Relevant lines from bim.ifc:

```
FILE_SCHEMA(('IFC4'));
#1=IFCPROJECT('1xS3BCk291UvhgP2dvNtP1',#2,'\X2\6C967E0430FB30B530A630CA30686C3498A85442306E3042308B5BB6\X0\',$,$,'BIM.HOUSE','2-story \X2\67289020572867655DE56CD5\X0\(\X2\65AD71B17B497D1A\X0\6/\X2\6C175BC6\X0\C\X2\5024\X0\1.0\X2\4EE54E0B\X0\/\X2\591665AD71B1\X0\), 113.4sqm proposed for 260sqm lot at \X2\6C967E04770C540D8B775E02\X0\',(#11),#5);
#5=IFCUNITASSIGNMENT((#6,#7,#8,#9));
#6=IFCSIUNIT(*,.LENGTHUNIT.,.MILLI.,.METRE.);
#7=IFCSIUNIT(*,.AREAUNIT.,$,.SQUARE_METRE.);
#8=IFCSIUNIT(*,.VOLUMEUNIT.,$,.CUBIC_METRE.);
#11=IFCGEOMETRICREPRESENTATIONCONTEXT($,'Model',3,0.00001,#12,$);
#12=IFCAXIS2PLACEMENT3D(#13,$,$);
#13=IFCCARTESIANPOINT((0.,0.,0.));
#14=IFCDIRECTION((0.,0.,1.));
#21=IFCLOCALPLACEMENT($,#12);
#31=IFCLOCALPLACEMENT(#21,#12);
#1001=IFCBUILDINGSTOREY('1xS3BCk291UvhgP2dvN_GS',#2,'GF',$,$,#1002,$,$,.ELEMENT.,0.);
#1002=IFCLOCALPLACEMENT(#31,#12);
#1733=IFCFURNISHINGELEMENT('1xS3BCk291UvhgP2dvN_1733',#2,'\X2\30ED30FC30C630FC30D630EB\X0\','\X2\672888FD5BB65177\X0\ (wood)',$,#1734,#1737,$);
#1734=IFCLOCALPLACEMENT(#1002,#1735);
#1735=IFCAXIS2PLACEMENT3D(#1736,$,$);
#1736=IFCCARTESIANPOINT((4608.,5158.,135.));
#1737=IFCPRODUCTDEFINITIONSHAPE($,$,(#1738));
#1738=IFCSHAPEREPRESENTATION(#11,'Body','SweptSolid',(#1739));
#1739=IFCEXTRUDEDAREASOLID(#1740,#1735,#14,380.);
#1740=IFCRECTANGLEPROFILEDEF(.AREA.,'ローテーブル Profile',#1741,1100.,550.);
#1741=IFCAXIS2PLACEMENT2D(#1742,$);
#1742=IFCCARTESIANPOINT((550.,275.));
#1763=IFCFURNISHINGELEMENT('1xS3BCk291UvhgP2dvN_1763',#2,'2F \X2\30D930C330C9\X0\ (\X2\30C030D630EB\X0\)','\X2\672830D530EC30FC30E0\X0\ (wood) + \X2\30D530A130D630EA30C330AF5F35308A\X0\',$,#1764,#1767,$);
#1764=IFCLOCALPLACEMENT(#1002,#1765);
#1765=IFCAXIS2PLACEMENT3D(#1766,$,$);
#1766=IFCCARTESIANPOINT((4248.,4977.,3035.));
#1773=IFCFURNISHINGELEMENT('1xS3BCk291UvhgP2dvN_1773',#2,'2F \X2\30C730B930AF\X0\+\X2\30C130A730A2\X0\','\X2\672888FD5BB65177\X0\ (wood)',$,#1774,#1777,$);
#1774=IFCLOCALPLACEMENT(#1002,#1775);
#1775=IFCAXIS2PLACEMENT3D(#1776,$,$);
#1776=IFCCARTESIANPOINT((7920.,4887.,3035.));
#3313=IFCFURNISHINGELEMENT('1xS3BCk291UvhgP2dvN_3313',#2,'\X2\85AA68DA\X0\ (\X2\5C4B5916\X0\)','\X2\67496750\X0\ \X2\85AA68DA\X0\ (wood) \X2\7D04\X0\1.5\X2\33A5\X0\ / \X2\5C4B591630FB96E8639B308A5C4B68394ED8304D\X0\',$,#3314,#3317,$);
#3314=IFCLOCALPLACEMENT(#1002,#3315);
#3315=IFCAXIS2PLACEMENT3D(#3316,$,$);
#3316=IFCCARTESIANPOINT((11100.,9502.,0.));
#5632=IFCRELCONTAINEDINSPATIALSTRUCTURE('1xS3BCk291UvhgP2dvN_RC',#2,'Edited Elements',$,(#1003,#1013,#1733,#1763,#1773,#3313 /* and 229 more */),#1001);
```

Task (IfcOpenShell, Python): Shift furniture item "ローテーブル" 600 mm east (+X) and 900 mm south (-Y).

```python
import ifcopenshell
import ifcopenshell.api.geometry
import ifcopenshell.util.placement
import ifcopenshell.util.unit

model = ifcopenshell.open("bim.ifc")
unit_scale = ifcopenshell.util.unit.calculate_unit_scale(model)

item = model.by_guid("1xS3BCk291UvhgP2dvN_1733")
matrix = ifcopenshell.util.placement.get_local_placement(item.ObjectPlacement)
matrix[0, 3] += 0.6 / unit_scale
matrix[1, 3] -= 0.9 / unit_scale
ifcopenshell.api.geometry.edit_object_placement(model, product=item, matrix=matrix, is_si=False)

print(ifcopenshell.util.placement.get_local_placement(item.ObjectPlacement).round(3) + 0.0)

model.write("bim_updated.ifc")
```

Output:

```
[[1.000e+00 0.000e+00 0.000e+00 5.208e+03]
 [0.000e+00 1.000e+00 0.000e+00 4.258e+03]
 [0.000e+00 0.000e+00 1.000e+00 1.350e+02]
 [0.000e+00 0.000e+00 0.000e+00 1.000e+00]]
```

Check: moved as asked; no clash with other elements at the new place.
